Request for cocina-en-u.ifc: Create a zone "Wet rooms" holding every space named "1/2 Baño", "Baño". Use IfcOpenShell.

First a look at what the model holds.

```python
import ifcopenshell

model = ifcopenshell.open("cocina-en-u.ifc")
print(model.schema)
seen = {}
for space in model.by_type("IfcSpace"):
    seen[space.LongName] = seen.get(space.LongName, 0) + 1
for name, count in sorted(seen.items(), key=str):
    print(count, "x", name)
print("zones:", [z.Name for z in model.by_type("IfcZone")][:20])
```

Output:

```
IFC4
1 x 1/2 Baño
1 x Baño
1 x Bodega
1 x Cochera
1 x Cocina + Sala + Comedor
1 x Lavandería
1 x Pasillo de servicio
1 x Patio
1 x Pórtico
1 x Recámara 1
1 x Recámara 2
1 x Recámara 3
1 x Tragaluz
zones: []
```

```python
import ifcopenshell
import ifcopenshell.api.group
import ifcopenshell.api.root

model = ifcopenshell.open("cocina-en-u.ifc")

names = {"1/2 Baño", "Baño"}
spaces = [s for s in model.by_type("IfcSpace") if s.LongName in names]

zone = ifcopenshell.api.root.create_entity(model, ifc_class="IfcZone", name="Wet rooms")
ifcopenshell.api.group.assign_group(model, products=spaces, group=zone)
print(len(spaces), "spaces in", zone.Name)

model.write("cocina-en-u_updated.ifc")
```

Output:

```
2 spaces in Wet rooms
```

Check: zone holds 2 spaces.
